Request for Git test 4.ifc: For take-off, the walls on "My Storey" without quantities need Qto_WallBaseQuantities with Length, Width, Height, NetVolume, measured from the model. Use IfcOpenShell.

First a look at what the model holds.

```python
import ifcopenshell
import ifcopenshell.util.element
import ifcopenshell.util.unit

model = ifcopenshell.open("Git test 4.ifc")
print(model.schema)
for unit_type in ("LENGTHUNIT", "AREAUNIT", "VOLUMEUNIT"):
    print(unit_type, ifcopenshell.util.unit.calculate_unit_scale(model, unit_type))
storey = next(s for s in model.by_type("IfcBuildingStorey") if s.Name == "My Storey")
walls = [e for e in ifcopenshell.util.element.get_decomposition(storey) if e.is_a("IfcWall")]
for e in sorted(walls, key=lambda e: e.id()):
    print(e.id(), e.is_a(), e.Name, list(ifcopenshell.util.element.get_psets(e, qtos_only=True)), sep=" | ")
```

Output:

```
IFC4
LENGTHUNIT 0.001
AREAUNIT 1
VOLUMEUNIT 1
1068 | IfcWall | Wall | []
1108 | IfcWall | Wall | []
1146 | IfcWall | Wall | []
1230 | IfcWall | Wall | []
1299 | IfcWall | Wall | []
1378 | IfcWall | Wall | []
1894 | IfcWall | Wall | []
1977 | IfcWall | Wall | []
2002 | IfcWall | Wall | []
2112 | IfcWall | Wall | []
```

```python
import ifcopenshell
import ifcopenshell.api.pset
import ifcopenshell.geom
import ifcopenshell.util.element
import ifcopenshell.util.shape
import ifcopenshell.util.unit

model = ifcopenshell.open("Git test 4.ifc")
unit_scale = ifcopenshell.util.unit.calculate_unit_scale(model)
volume_scale = ifcopenshell.util.unit.calculate_unit_scale(model, "VOLUMEUNIT")
settings = ifcopenshell.geom.settings()

storey = next(s for s in model.by_type("IfcBuildingStorey") if s.Name == "My Storey")
walls = [e for e in ifcopenshell.util.element.get_decomposition(storey) if e.is_a("IfcWall")]

for e in sorted(walls, key=lambda e: e.id()):
    if ifcopenshell.util.element.get_psets(e, qtos_only=True, should_inherit=False):
        continue
    # Geometry comes back in metres, in the element's own axes.
    shape = ifcopenshell.geom.create_shape(settings, e)
    values = {
        "Length": ifcopenshell.util.shape.get_x(shape.geometry) / unit_scale,
        "Width": ifcopenshell.util.shape.get_y(shape.geometry) / unit_scale,
        "Height": ifcopenshell.util.shape.get_z(shape.geometry) / unit_scale,
        "NetVolume": ifcopenshell.util.shape.get_volume(shape.geometry) / volume_scale,
    }
    qto = ifcopenshell.api.pset.add_qto(model, product=e, name="Qto_WallBaseQuantities")
    ifcopenshell.api.pset.edit_qto(model, qto=qto, properties=values)
    print(e.id(), {k: round(v, 3) for k, v in values.items()})

model.write("Git test 4_edited.ifc")
```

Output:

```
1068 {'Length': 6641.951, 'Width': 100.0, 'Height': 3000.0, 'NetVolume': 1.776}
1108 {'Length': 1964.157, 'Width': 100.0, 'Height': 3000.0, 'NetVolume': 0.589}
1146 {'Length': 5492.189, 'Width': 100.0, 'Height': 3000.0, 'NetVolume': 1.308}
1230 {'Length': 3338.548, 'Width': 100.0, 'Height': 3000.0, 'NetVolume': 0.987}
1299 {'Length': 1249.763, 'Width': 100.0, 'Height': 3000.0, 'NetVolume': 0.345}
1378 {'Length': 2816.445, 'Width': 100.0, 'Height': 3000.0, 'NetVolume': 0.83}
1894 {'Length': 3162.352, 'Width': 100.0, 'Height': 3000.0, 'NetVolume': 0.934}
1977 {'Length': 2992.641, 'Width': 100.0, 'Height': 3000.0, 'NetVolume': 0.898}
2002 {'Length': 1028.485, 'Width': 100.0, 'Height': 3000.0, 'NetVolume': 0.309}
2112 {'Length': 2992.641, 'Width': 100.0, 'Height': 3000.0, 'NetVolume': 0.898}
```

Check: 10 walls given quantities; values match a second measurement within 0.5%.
